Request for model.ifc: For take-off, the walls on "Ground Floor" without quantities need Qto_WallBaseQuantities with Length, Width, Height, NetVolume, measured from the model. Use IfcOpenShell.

First a look at what the model holds.

```python
import ifcopenshell
import ifcopenshell.util.element
import ifcopenshell.util.unit

model = ifcopenshell.open("model.ifc")
print(model.schema)
for unit_type in ("LENGTHUNIT", "AREAUNIT", "VOLUMEUNIT"):
    print(unit_type, ifcopenshell.util.unit.calculate_unit_scale(model, unit_type))
storey = next(s for s in model.by_type("IfcBuildingStorey") if s.Name == "Ground Floor")
walls = [e for e in ifcopenshell.util.element.get_decomposition(storey) if e.is_a("IfcWall")]
for e in sorted(walls, key=lambda e: e.id()):
    print(e.id(), e.is_a(), e.Name, list(ifcopenshell.util.element.get_psets(e, qtos_only=True)), sep=" | ")
```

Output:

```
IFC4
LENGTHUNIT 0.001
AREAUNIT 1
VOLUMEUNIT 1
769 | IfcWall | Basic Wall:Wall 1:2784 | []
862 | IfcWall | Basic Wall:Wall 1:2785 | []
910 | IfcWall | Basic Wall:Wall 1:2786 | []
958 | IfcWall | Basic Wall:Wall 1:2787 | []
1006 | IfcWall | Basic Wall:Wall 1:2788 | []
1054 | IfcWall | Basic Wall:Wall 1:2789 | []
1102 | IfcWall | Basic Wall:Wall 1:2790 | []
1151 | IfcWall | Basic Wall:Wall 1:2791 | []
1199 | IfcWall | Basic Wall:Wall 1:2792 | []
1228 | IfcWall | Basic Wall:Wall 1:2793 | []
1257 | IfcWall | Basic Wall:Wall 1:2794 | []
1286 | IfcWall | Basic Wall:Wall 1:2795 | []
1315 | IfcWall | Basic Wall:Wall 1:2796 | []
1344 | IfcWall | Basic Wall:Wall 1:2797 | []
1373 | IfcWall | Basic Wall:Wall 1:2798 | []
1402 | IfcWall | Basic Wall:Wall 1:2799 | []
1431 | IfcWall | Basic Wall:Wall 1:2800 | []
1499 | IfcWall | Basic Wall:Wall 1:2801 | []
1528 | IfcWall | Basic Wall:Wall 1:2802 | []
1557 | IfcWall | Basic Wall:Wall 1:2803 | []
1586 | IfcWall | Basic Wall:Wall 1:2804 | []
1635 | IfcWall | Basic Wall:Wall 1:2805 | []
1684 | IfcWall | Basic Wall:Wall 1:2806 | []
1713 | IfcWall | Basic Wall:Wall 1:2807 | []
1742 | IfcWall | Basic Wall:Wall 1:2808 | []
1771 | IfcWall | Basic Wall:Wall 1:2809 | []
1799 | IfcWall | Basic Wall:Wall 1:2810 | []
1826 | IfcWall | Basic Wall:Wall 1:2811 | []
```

```python
import ifcopenshell
import ifcopenshell.api.pset
import ifcopenshell.geom
import ifcopenshell.util.element
import ifcopenshell.util.shape
import ifcopenshell.util.unit

model = ifcopenshell.open("model.ifc")
unit_scale = ifcopenshell.util.unit.calculate_unit_scale(model)
volume_scale = ifcopenshell.util.unit.calculate_unit_scale(model, "VOLUMEUNIT")
settings = ifcopenshell.geom.settings()

storey = next(s for s in model.by_type("IfcBuildingStorey") if s.Name == "Ground Floor")
walls = [e for e in ifcopenshell.util.element.get_decomposition(storey) if e.is_a("IfcWall")]

for e in sorted(walls, key=lambda e: e.id()):
    if ifcopenshell.util.element.get_psets(e, qtos_only=True, should_inherit=False):
        continue
    # Geometry comes back in metres, in the element's own axes.
    shape = ifcopenshell.geom.create_shape(settings, e)
    values = {
        "Length": ifcopenshell.util.shape.get_x(shape.geometry) / unit_scale,
        "Width": ifcopenshell.util.shape.get_y(shape.geometry) / unit_scale,
        "Height": ifcopenshell.util.shape.get_z(shape.geometry) / unit_scale,
        "NetVolume": ifcopenshell.util.shape.get_volume(shape.geometry) / volume_scale,
    }
    qto = ifcopenshell.api.pset.add_qto(model, product=e, name="Qto_WallBaseQuantities")
    ifcopenshell.api.pset.edit_qto(model, qto=qto, properties=values)
    print(e.id(), {k: round(v, 3) for k, v in values.items()})

model.write("model_updated.ifc")
```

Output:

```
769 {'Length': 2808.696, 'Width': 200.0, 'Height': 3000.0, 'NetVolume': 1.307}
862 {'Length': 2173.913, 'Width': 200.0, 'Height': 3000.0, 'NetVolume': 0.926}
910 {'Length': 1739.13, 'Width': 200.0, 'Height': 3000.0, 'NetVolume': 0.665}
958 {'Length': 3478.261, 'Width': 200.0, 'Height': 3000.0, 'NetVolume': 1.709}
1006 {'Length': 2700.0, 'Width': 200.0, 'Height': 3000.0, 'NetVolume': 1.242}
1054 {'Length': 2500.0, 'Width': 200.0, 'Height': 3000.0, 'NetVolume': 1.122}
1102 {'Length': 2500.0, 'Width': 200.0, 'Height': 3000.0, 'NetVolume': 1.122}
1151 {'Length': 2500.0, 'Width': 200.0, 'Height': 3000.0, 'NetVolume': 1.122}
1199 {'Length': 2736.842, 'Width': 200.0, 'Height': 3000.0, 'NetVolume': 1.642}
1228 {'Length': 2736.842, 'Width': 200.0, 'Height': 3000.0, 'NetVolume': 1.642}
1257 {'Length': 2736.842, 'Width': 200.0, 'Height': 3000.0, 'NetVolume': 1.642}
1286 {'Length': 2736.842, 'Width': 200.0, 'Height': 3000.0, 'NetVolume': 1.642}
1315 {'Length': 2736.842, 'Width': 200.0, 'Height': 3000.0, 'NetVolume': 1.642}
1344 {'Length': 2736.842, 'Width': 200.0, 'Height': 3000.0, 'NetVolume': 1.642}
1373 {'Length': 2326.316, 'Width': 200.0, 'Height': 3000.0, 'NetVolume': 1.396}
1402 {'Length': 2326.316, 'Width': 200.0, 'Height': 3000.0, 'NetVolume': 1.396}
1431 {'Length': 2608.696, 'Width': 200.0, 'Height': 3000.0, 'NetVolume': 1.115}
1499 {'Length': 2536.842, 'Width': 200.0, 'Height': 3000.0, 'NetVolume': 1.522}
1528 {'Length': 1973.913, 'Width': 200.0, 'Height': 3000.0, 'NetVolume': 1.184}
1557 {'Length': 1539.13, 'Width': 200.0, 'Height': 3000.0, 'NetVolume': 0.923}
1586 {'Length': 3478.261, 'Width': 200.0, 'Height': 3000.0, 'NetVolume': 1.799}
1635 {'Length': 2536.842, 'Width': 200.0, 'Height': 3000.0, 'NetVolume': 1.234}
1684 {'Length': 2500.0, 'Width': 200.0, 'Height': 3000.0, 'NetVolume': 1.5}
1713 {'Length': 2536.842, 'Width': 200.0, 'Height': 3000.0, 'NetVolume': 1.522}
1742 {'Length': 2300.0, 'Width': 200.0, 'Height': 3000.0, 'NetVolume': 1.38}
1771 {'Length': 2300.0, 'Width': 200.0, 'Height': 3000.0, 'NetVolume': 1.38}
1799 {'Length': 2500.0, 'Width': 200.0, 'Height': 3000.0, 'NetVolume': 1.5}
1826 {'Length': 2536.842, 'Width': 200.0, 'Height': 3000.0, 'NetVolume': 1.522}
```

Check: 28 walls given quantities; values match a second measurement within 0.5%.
